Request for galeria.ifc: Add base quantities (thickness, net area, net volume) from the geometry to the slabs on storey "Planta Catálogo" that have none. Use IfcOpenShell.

First a look at what the model holds.

```python
import ifcopenshell
import ifcopenshell.util.element
import ifcopenshell.util.unit

model = ifcopenshell.open("galeria.ifc")
print(model.schema)
for unit_type in ("LENGTHUNIT", "AREAUNIT", "VOLUMEUNIT"):
    print(unit_type, ifcopenshell.util.unit.calculate_unit_scale(model, unit_type))
storey = next(s for s in model.by_type("IfcBuildingStorey") if s.Name == "Planta Catálogo")
slabs = [e for e in ifcopenshell.util.element.get_decomposition(storey) if e.is_a("IfcSlab")]
for e in sorted(slabs, key=lambda e: e.id()):
    print(e.id(), e.is_a(), e.Name, list(ifcopenshell.util.element.get_psets(e, qtos_only=True)), sep=" | ")
```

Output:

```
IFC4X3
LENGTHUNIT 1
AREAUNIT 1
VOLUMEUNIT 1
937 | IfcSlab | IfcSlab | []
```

```python
import ifcopenshell
import ifcopenshell.api.pset
import ifcopenshell.geom
import ifcopenshell.util.element
import ifcopenshell.util.shape
import ifcopenshell.util.unit

model = ifcopenshell.open("galeria.ifc")
unit_scale = ifcopenshell.util.unit.calculate_unit_scale(model)
area_scale = ifcopenshell.util.unit.calculate_unit_scale(model, "AREAUNIT")
volume_scale = ifcopenshell.util.unit.calculate_unit_scale(model, "VOLUMEUNIT")
settings = ifcopenshell.geom.settings()

storey = next(s for s in model.by_type("IfcBuildingStorey") if s.Name == "Planta Catálogo")
slabs = [e for e in ifcopenshell.util.element.get_decomposition(storey) if e.is_a("IfcSlab")]

for e in sorted(slabs, key=lambda e: e.id()):
    if ifcopenshell.util.element.get_psets(e, qtos_only=True, should_inherit=False):
        continue
    # Geometry comes back in metres, in the element's own axes.
    shape = ifcopenshell.geom.create_shape(settings, e)
    values = {
        "Width": ifcopenshell.util.shape.get_z(shape.geometry) / unit_scale,
        "NetArea": ifcopenshell.util.shape.get_footprint_area(shape.geometry) / area_scale,
        "NetVolume": ifcopenshell.util.shape.get_volume(shape.geometry) / volume_scale,
    }
    qto = ifcopenshell.api.pset.add_qto(model, product=e, name="Qto_SlabBaseQuantities")
    ifcopenshell.api.pset.edit_qto(model, qto=qto, properties=values)
    print(e.id(), {k: round(v, 3) for k, v in values.items()})

model.write("galeria-out.ifc")
```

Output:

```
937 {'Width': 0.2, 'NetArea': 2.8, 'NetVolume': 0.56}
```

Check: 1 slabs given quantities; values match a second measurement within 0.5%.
